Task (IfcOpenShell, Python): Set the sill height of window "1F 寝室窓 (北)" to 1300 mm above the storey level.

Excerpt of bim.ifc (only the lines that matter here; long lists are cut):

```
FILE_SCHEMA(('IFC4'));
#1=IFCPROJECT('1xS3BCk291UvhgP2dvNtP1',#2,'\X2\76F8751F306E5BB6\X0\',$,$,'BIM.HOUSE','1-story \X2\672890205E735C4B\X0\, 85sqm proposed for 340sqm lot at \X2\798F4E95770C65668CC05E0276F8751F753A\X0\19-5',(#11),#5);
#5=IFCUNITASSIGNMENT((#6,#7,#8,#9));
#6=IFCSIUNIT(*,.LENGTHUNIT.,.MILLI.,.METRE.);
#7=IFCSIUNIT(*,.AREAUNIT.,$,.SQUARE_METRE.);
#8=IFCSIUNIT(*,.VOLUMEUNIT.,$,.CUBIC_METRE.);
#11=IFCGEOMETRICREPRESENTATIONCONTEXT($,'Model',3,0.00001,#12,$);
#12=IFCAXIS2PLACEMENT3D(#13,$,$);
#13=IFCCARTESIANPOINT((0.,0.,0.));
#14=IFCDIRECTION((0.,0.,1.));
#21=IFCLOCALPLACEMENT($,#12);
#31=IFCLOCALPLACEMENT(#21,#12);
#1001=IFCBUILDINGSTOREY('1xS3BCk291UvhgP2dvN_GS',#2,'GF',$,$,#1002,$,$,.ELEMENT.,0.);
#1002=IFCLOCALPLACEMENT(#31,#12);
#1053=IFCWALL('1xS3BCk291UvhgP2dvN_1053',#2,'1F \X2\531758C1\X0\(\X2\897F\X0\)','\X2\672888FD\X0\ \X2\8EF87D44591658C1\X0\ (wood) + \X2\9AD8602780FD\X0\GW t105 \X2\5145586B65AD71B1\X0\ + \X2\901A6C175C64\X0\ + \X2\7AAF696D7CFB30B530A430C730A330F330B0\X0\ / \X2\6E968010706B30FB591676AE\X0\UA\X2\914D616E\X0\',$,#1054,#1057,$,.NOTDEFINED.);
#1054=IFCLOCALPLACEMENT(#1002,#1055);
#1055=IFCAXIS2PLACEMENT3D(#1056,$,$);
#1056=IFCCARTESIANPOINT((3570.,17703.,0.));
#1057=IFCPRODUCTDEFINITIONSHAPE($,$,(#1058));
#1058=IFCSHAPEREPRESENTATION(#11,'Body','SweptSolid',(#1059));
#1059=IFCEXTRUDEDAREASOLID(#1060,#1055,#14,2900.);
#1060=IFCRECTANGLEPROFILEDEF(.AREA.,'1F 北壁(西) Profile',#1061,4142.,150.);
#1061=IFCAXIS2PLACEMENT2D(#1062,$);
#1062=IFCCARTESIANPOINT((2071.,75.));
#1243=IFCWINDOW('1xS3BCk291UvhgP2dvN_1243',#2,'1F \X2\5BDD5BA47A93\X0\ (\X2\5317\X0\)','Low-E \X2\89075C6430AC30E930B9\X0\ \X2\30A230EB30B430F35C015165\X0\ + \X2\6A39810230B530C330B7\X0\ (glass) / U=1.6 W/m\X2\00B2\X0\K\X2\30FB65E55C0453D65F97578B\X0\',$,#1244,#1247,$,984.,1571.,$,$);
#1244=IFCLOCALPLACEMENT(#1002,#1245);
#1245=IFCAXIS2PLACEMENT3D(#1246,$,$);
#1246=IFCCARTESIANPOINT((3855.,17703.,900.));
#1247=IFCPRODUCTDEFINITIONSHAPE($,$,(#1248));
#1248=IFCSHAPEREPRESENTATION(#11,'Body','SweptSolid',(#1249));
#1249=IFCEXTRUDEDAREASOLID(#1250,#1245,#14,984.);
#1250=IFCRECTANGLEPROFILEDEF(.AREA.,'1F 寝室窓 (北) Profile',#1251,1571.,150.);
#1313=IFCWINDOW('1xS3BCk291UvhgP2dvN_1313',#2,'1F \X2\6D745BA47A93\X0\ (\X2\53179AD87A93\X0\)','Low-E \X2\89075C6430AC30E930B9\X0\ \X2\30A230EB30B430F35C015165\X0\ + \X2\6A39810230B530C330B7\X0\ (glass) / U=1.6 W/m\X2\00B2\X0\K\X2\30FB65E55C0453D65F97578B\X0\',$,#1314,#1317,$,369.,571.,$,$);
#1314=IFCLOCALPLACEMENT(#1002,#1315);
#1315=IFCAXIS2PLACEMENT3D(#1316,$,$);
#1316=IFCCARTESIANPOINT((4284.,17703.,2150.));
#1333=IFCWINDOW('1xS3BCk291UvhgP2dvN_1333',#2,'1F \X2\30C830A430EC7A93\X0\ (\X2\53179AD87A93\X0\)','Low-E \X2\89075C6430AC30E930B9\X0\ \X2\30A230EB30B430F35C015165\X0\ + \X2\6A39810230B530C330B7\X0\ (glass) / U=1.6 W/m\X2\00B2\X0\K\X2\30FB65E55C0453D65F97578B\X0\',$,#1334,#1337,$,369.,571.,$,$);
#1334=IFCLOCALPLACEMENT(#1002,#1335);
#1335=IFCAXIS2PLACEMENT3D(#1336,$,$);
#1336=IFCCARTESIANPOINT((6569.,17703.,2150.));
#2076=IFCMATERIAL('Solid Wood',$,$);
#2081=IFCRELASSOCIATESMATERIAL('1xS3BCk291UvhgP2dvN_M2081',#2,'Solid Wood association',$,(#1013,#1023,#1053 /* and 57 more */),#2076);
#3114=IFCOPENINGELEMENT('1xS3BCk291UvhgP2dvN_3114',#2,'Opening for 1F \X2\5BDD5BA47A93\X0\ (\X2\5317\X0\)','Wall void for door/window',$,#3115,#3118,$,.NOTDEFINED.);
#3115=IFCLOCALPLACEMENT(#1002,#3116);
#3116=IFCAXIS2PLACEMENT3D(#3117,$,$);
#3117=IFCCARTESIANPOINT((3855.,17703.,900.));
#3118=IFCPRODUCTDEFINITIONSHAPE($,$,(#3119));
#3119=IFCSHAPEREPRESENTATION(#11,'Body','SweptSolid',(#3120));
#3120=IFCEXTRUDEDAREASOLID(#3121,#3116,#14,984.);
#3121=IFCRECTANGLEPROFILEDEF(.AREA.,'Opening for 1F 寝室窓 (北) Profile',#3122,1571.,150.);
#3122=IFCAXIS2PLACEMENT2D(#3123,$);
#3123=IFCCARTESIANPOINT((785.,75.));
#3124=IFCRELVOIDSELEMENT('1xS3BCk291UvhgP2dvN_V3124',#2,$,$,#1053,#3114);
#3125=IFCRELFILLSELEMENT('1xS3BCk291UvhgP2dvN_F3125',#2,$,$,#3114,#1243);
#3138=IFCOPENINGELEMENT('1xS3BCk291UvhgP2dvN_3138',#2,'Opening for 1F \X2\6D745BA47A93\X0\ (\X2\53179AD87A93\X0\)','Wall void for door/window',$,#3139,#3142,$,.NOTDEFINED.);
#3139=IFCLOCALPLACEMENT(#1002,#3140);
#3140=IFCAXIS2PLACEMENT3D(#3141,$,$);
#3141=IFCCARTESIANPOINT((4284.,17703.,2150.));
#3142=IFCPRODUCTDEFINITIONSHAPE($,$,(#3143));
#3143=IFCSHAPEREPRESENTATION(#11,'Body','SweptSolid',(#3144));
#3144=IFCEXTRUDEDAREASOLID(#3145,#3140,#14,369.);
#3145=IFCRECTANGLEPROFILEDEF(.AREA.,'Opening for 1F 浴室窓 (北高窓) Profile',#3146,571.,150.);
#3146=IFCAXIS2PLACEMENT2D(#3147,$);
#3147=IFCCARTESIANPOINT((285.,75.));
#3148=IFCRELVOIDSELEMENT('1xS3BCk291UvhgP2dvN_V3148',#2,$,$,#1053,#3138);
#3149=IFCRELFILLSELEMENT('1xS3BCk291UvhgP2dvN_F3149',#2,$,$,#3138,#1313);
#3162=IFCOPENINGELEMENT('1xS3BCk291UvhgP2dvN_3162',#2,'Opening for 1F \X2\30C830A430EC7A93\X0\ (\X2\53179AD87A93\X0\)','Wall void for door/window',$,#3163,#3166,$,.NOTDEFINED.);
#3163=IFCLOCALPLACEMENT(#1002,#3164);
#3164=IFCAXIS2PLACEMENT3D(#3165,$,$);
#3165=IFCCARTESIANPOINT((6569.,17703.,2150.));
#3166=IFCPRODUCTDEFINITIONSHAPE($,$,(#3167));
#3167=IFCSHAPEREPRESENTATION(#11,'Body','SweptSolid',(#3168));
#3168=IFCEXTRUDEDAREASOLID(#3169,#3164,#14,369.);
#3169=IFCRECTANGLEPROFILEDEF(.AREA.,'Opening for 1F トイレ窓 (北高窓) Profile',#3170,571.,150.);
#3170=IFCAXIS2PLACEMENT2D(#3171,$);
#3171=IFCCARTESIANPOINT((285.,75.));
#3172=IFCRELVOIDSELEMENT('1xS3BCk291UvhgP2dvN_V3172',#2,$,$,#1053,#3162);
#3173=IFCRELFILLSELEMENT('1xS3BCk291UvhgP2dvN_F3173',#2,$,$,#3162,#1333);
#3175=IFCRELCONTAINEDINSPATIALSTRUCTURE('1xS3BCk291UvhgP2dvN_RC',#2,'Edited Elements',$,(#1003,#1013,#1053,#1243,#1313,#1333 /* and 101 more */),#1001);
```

```python
import numpy as np
import ifcopenshell
import ifcopenshell.api.geometry
import ifcopenshell.geom
import ifcopenshell.util.element
import ifcopenshell.util.placement
import ifcopenshell.util.shape
import ifcopenshell.util.unit

model = ifcopenshell.open("bim.ifc")
unit_scale = ifcopenshell.util.unit.calculate_unit_scale(model)

window = model.by_guid("1xS3BCk291UvhgP2dvN_1243")
opening = window.FillsVoids[0].RelatingOpeningElement
storey = ifcopenshell.util.element.get_container(window, ifc_class="IfcBuildingStorey")
level = ifcopenshell.util.placement.get_local_placement(storey.ObjectPlacement)[2, 3]

# The opening's origin need not be at the sill, so measure its lowest point.
shape = ifcopenshell.geom.create_shape(ifcopenshell.geom.settings(), opening)
bottom = ifcopenshell.util.shape.get_shape_bottom_elevation(shape, shape.geometry) / unit_scale
dz = level + 1.3 / unit_scale - bottom

shift = np.array([0.0, 0.0, dz])
# The window is not placed relative to its opening, so move both.
for product in (opening, window):
    matrix = ifcopenshell.util.placement.get_local_placement(product.ObjectPlacement)
    matrix[:3, 3] += shift
    ifcopenshell.api.geometry.edit_object_placement(model, product=product, matrix=matrix, is_si=False)

print(f"moved by {dz * unit_scale:+.3f} m")

model.write("bim_edited.ifc")
```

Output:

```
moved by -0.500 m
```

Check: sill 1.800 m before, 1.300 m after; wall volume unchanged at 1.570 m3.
